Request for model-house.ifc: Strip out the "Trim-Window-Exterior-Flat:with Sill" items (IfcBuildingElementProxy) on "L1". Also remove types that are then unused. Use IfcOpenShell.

First a look at what the model holds.

```python
import ifcopenshell
import ifcopenshell.util.element

model = ifcopenshell.open("model-house.ifc")
print(model.schema)
storey = next(s for s in model.by_type("IfcBuildingStorey") if s.Name == "L1")
proxies = [e for e in ifcopenshell.util.element.get_decomposition(storey) if e.is_a("IfcBuildingElementProxy")]
seen = {}
for e in proxies:
    element_type = ifcopenshell.util.element.get_type(e)
    name = element_type.Name if element_type not in (None, e) else None
    seen[name] = seen.get(name, 0) + 1
for name, count in sorted(seen.items(), key=str):
    print(count, "x", name)
```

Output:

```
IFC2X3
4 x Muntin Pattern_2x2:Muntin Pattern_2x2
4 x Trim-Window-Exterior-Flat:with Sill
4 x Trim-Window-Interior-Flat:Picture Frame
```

```python
import ifcopenshell
import ifcopenshell.api.root
import ifcopenshell.util.element

model = ifcopenshell.open("model-house.ifc")

storey = next(s for s in model.by_type("IfcBuildingStorey") if s.Name == "L1")
proxies = [e for e in ifcopenshell.util.element.get_decomposition(storey) if e.is_a("IfcBuildingElementProxy")]
targets = [e for e in proxies if (t := ifcopenshell.util.element.get_type(e)) not in (None, e) and t.Name == "Trim-Window-Exterior-Flat:with Sill"]
types = {ifcopenshell.util.element.get_type(e) for e in targets} - {None, *targets}

for e in targets:
    ifcopenshell.api.root.remove_product(model, product=e)
print(len(targets), "removed")

unused = [t for t in types if not ifcopenshell.util.element.get_types(t)]
for t in unused:
    ifcopenshell.api.root.remove_product(model, product=t)
print(len(unused), "unused types removed")

model.write("model-house_updated.ifc")
```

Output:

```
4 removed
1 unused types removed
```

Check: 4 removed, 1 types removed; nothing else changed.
